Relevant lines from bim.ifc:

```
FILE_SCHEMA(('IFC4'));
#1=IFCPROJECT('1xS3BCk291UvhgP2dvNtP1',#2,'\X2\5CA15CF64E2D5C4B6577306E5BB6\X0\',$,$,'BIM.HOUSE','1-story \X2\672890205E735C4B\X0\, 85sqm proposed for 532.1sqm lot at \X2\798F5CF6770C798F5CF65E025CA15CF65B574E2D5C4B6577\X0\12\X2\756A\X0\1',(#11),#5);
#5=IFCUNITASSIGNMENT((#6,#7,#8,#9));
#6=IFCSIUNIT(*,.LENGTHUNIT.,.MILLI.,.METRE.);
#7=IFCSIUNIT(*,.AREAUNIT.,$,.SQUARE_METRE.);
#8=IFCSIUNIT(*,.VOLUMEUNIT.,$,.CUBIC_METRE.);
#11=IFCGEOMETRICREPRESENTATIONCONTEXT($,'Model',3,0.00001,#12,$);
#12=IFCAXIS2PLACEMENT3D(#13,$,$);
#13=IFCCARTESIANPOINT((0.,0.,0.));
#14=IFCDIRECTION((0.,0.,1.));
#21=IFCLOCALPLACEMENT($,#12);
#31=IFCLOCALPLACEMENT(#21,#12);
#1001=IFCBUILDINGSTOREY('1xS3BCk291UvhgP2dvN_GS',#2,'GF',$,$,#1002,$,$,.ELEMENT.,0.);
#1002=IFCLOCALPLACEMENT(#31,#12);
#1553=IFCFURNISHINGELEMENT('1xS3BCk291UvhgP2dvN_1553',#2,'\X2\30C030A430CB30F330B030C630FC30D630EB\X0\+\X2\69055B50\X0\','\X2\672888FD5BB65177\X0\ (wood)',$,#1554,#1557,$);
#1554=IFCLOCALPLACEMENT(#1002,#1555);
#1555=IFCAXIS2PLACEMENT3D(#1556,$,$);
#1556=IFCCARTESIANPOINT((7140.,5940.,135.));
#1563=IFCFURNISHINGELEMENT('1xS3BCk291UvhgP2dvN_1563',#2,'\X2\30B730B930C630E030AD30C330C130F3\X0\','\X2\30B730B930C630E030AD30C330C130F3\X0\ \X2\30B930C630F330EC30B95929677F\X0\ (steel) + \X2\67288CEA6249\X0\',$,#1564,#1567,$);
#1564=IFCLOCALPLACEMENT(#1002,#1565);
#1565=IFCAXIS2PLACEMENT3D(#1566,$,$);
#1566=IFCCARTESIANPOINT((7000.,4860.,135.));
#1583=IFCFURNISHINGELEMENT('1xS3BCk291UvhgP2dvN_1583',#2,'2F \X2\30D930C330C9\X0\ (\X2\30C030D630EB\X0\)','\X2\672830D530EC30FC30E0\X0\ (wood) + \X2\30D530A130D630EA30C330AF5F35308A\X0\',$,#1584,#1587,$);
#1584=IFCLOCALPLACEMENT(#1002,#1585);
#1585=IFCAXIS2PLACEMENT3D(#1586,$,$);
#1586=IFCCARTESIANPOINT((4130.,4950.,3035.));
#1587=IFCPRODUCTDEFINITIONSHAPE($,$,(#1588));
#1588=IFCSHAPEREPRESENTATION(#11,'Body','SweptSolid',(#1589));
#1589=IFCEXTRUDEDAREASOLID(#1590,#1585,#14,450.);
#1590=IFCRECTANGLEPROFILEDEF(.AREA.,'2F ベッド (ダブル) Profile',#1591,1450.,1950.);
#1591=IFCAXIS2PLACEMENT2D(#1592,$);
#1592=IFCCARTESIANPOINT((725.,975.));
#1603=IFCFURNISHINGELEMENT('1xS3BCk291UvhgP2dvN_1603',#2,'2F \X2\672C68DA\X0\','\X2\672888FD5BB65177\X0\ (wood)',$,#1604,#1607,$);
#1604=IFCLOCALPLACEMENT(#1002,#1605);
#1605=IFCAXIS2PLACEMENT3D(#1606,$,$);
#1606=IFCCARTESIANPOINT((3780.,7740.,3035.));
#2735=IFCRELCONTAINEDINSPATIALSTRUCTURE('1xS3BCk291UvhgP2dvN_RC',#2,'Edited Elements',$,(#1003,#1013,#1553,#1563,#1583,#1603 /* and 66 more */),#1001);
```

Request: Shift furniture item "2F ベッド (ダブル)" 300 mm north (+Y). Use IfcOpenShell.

```python
import ifcopenshell
import ifcopenshell.api.geometry
import ifcopenshell.util.placement
import ifcopenshell.util.unit

model = ifcopenshell.open("bim.ifc")
unit_scale = ifcopenshell.util.unit.calculate_unit_scale(model)

item = model.by_guid("1xS3BCk291UvhgP2dvN_1583")
matrix = ifcopenshell.util.placement.get_local_placement(item.ObjectPlacement)
matrix[1, 3] += 0.3 / unit_scale
ifcopenshell.api.geometry.edit_object_placement(model, product=item, matrix=matrix, is_si=False)

print(ifcopenshell.util.placement.get_local_placement(item.ObjectPlacement).round(3) + 0.0)

model.write("bim_v2.ifc")
```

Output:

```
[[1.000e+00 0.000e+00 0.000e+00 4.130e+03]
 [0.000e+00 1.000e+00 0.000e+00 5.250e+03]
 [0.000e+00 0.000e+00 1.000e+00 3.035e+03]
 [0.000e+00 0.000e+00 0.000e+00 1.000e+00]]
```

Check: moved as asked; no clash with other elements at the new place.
